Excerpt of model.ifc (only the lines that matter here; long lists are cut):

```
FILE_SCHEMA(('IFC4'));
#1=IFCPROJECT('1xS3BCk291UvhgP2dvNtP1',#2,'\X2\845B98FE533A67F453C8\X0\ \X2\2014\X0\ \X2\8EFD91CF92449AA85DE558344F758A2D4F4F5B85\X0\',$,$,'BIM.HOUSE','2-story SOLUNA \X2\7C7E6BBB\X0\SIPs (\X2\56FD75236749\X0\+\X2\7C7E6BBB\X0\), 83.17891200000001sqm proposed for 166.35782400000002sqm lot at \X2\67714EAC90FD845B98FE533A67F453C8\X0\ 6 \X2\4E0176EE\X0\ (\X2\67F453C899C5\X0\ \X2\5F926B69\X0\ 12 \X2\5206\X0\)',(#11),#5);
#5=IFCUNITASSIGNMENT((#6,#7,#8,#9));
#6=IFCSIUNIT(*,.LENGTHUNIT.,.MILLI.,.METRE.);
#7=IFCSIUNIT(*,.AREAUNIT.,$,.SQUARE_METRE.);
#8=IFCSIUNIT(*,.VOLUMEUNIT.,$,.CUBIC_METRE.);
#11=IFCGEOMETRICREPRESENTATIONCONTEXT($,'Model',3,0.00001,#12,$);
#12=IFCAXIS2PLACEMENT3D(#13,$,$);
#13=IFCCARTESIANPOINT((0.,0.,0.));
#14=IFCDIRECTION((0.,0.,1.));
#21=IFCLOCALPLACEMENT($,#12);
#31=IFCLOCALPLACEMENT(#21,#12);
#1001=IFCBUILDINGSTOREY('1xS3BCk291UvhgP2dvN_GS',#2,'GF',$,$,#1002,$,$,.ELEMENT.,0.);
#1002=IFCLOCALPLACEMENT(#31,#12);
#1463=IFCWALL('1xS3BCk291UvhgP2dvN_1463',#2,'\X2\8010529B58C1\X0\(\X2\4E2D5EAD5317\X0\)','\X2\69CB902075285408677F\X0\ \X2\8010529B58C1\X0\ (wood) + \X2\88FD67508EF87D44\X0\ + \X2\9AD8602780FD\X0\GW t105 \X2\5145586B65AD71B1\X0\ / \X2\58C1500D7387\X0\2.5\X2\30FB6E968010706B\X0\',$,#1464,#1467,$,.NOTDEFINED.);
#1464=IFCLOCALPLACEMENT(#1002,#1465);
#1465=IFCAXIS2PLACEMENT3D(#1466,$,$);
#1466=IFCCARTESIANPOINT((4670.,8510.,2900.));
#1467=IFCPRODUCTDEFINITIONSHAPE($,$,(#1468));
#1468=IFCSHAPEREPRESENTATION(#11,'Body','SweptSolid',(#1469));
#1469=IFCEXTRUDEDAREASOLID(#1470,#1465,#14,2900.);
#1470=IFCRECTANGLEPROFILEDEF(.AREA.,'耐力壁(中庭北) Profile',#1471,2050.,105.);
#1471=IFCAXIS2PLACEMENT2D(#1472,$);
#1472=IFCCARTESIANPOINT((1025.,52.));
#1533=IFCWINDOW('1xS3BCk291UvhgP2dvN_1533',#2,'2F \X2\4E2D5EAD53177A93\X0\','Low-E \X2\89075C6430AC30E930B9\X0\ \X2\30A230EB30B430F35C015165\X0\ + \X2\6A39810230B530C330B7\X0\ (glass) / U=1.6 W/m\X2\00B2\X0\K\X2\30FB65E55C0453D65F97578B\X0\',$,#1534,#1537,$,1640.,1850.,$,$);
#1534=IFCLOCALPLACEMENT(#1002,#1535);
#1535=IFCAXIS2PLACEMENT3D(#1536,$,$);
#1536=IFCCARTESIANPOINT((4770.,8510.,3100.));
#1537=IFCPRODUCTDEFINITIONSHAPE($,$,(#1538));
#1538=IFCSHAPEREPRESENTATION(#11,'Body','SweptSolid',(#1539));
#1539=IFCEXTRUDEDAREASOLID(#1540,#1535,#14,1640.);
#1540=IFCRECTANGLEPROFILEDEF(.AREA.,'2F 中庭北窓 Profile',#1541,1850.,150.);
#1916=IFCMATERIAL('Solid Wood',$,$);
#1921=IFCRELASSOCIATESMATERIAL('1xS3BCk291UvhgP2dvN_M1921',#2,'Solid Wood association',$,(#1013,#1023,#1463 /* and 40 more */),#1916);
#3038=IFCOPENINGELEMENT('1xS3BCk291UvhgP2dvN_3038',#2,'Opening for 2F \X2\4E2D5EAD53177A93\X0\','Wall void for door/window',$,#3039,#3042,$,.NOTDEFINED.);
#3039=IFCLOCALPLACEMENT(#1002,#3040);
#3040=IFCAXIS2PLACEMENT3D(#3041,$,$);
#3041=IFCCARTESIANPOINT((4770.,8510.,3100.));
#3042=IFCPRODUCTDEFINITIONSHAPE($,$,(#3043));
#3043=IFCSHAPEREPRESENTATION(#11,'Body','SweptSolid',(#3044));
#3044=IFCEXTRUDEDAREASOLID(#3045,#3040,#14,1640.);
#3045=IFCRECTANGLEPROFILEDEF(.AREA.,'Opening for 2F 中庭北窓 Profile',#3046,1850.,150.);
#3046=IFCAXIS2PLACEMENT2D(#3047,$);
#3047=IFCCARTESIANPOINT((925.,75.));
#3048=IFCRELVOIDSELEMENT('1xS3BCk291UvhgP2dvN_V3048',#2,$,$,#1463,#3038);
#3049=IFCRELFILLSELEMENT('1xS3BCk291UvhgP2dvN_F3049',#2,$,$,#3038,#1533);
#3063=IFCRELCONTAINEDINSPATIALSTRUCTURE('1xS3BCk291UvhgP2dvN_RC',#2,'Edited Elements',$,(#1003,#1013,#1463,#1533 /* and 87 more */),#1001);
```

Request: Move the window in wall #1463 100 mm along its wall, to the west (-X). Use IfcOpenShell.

```python
import ifcopenshell
import ifcopenshell.api.geometry
import ifcopenshell.util.placement
import ifcopenshell.util.unit

model = ifcopenshell.open("model.ifc")
unit_scale = ifcopenshell.util.unit.calculate_unit_scale(model)

window = model.by_guid("1xS3BCk291UvhgP2dvN_1533")
opening = window.FillsVoids[0].RelatingOpeningElement
wall = opening.VoidsElements[0].RelatingBuildingElement

wall_matrix = ifcopenshell.util.placement.get_local_placement(wall.ObjectPlacement)
shift = wall_matrix[:3, 0] * -0.1 / unit_scale
before = ifcopenshell.util.placement.get_local_placement(window.ObjectPlacement)[:3, 3].copy()

# The window is not placed relative to its opening, so move both.
for product in (opening, window):
    matrix = ifcopenshell.util.placement.get_local_placement(product.ObjectPlacement)
    matrix[:3, 3] += shift
    ifcopenshell.api.geometry.edit_object_placement(model, product=product, matrix=matrix, is_si=False)

after = ifcopenshell.util.placement.get_local_placement(window.ObjectPlacement)[:3, 3]
print("window moved by", (after - before).round(3) + 0.0)

model.write("model_updated.ifc")
```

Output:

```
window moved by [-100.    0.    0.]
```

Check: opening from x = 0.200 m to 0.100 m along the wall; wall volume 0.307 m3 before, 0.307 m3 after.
